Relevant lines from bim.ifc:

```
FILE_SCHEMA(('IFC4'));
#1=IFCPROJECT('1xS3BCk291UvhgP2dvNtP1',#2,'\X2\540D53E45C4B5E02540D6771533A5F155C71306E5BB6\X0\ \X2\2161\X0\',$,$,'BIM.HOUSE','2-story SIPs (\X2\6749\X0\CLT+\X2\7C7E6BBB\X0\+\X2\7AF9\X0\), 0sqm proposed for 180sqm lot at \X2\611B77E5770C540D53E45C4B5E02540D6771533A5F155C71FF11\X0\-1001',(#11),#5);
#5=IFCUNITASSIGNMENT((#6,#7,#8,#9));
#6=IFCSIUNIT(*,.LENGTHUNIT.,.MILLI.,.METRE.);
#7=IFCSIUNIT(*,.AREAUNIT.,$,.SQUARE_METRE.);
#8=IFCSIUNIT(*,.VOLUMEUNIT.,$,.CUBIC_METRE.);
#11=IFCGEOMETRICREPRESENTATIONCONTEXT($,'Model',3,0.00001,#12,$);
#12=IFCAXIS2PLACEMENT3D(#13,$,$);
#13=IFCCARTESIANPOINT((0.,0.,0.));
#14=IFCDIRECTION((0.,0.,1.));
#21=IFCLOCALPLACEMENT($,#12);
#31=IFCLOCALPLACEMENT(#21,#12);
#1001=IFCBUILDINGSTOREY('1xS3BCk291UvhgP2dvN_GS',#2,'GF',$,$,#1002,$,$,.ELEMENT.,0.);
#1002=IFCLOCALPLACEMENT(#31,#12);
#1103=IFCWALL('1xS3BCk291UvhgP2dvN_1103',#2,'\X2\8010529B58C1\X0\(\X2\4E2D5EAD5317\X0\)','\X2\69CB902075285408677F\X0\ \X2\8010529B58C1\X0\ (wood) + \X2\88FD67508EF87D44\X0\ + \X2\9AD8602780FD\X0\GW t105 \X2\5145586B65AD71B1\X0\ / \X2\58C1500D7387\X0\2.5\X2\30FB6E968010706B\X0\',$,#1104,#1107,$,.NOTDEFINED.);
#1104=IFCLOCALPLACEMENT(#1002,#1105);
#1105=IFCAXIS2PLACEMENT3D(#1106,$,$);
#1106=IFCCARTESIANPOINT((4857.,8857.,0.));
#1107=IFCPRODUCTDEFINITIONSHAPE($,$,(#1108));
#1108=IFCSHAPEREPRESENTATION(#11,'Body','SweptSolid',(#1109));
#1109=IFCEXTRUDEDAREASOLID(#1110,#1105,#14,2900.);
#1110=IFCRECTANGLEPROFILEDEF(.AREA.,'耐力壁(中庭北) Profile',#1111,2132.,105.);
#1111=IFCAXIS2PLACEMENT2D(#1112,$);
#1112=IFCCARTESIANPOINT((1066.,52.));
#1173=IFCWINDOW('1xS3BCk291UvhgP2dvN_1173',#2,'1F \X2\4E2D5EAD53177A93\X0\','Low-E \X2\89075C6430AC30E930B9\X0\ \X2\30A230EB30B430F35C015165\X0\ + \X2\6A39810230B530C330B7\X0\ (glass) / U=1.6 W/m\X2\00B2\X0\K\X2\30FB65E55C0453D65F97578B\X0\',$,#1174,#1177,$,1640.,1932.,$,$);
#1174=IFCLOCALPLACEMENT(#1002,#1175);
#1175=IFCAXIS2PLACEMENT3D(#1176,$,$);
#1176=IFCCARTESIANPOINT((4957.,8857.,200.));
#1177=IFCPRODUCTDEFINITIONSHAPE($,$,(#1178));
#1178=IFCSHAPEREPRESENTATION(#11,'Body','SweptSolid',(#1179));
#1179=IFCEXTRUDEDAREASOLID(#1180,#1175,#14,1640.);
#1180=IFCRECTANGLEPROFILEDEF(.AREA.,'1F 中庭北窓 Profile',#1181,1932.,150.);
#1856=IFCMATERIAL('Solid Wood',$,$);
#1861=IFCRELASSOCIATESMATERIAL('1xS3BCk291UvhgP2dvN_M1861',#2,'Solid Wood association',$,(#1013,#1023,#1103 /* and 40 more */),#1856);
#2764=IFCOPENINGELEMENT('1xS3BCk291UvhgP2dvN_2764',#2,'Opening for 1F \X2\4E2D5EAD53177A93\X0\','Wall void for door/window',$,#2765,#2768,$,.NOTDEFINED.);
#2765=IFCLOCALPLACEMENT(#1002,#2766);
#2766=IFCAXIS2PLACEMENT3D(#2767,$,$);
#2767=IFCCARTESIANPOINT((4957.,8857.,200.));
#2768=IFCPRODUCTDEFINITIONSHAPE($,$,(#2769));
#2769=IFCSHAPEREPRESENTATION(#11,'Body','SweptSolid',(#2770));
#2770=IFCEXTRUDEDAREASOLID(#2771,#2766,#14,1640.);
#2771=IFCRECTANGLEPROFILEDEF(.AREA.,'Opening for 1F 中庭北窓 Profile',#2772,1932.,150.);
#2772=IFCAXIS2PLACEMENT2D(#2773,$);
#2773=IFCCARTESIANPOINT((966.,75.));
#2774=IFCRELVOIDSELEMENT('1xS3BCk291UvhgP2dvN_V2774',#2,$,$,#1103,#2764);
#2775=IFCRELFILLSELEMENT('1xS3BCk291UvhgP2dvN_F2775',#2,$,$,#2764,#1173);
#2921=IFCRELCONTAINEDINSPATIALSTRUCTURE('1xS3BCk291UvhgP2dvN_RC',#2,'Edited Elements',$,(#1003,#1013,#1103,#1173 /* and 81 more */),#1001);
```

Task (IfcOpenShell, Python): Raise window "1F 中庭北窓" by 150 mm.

```python
import numpy as np
import ifcopenshell
import ifcopenshell.api.geometry
import ifcopenshell.util.placement
import ifcopenshell.util.unit

model = ifcopenshell.open("bim.ifc")
unit_scale = ifcopenshell.util.unit.calculate_unit_scale(model)

window = model.by_guid("1xS3BCk291UvhgP2dvN_1173")
opening = window.FillsVoids[0].RelatingOpeningElement
dz = 0.15 / unit_scale

shift = np.array([0.0, 0.0, dz])
# The window is not placed relative to its opening, so move both.
for product in (opening, window):
    matrix = ifcopenshell.util.placement.get_local_placement(product.ObjectPlacement)
    matrix[:3, 3] += shift
    ifcopenshell.api.geometry.edit_object_placement(model, product=product, matrix=matrix, is_si=False)

print(f"moved by {dz * unit_scale:+.3f} m")

model.write("bim_edited.ifc")
```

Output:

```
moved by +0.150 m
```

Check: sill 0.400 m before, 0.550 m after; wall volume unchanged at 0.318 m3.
